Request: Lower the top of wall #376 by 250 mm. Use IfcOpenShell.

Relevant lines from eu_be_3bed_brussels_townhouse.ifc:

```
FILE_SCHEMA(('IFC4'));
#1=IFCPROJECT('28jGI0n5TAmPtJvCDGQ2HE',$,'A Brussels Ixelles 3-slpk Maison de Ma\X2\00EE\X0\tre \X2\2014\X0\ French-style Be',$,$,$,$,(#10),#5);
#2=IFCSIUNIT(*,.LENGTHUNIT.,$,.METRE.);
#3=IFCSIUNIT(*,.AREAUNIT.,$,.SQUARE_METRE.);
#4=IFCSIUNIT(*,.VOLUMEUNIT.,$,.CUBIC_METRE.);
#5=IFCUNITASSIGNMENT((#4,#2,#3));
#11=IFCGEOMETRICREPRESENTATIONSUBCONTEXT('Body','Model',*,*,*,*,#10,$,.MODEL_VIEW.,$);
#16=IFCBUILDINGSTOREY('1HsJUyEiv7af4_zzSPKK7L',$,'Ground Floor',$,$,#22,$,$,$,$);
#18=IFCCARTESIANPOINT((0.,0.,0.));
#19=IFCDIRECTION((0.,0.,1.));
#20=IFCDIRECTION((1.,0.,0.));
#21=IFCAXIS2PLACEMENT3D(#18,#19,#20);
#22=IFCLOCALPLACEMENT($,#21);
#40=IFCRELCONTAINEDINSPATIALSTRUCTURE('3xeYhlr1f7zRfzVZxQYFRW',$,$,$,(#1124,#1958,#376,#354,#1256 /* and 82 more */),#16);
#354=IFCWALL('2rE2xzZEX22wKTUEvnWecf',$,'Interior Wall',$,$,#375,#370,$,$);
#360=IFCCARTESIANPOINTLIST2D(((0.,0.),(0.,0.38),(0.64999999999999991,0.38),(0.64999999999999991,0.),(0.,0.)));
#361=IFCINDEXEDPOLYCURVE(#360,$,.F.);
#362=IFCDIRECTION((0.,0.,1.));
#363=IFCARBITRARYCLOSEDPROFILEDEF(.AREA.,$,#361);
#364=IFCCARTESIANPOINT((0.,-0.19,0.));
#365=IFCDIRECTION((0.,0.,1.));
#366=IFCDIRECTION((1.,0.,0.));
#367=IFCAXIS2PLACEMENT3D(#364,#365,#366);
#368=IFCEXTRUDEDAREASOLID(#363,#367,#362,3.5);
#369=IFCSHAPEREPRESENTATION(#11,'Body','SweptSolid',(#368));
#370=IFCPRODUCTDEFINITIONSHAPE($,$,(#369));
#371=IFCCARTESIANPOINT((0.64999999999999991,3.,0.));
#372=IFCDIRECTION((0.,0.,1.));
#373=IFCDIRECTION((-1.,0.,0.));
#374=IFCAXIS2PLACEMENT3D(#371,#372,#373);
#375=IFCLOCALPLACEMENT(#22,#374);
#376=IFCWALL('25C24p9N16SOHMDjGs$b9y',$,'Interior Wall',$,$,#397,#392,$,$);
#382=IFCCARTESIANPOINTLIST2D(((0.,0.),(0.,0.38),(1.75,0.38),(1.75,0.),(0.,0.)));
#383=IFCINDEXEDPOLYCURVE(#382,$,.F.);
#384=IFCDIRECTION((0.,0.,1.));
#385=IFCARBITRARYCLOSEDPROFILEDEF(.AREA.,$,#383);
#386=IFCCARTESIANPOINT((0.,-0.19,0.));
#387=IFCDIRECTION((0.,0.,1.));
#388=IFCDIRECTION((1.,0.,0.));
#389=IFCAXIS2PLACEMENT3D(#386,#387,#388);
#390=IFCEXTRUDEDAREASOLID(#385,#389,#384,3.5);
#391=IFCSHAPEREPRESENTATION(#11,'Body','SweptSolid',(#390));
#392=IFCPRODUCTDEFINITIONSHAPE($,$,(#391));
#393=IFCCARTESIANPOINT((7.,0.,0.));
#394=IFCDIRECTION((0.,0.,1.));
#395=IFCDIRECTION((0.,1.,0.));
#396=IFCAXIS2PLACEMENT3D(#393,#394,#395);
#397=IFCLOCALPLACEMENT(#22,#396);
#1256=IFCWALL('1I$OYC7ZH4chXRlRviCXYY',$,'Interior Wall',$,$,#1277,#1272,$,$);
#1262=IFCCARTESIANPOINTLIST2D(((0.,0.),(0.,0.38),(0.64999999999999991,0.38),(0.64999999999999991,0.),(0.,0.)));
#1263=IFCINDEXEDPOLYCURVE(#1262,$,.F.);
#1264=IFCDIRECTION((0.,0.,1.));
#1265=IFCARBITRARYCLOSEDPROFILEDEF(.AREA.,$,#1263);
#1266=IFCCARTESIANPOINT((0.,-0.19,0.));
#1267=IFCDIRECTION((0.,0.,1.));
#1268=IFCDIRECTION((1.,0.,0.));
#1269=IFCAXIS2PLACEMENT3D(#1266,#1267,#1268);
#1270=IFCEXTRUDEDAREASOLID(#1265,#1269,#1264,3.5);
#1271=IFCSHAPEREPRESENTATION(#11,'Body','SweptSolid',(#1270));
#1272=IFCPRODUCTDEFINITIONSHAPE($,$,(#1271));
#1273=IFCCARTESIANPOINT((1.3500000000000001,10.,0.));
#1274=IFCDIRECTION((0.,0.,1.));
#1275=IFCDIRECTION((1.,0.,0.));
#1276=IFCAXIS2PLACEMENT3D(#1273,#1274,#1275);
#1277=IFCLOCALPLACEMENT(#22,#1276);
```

```python
import ifcopenshell
import ifcopenshell.geom
import ifcopenshell.util.representation
import ifcopenshell.util.shape

model = ifcopenshell.open("eu_be_3bed_brussels_townhouse.ifc")
settings = ifcopenshell.geom.settings()


def volume(element):
    """Net volume in cubic metres, openings subtracted."""
    shape = ifcopenshell.geom.create_shape(settings, element)
    return ifcopenshell.util.shape.get_volume(shape.geometry)


wall = model.by_guid("25C24p9N16SOHMDjGs$b9y")
before = volume(wall)

body = ifcopenshell.util.representation.get_representation(wall, "Model", "Body")
solid = body.Items[0]
old_height = solid.Depth
solid.Depth -= 0.25
after = volume(wall)

print(f"height {old_height:g} -> {solid.Depth:g}, volume {before:.3f} -> {after:.3f} m3")

model.write("eu_be_3bed_brussels_townhouse_edited.ifc")
```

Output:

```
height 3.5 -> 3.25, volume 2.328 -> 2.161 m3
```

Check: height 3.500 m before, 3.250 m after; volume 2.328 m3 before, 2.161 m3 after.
